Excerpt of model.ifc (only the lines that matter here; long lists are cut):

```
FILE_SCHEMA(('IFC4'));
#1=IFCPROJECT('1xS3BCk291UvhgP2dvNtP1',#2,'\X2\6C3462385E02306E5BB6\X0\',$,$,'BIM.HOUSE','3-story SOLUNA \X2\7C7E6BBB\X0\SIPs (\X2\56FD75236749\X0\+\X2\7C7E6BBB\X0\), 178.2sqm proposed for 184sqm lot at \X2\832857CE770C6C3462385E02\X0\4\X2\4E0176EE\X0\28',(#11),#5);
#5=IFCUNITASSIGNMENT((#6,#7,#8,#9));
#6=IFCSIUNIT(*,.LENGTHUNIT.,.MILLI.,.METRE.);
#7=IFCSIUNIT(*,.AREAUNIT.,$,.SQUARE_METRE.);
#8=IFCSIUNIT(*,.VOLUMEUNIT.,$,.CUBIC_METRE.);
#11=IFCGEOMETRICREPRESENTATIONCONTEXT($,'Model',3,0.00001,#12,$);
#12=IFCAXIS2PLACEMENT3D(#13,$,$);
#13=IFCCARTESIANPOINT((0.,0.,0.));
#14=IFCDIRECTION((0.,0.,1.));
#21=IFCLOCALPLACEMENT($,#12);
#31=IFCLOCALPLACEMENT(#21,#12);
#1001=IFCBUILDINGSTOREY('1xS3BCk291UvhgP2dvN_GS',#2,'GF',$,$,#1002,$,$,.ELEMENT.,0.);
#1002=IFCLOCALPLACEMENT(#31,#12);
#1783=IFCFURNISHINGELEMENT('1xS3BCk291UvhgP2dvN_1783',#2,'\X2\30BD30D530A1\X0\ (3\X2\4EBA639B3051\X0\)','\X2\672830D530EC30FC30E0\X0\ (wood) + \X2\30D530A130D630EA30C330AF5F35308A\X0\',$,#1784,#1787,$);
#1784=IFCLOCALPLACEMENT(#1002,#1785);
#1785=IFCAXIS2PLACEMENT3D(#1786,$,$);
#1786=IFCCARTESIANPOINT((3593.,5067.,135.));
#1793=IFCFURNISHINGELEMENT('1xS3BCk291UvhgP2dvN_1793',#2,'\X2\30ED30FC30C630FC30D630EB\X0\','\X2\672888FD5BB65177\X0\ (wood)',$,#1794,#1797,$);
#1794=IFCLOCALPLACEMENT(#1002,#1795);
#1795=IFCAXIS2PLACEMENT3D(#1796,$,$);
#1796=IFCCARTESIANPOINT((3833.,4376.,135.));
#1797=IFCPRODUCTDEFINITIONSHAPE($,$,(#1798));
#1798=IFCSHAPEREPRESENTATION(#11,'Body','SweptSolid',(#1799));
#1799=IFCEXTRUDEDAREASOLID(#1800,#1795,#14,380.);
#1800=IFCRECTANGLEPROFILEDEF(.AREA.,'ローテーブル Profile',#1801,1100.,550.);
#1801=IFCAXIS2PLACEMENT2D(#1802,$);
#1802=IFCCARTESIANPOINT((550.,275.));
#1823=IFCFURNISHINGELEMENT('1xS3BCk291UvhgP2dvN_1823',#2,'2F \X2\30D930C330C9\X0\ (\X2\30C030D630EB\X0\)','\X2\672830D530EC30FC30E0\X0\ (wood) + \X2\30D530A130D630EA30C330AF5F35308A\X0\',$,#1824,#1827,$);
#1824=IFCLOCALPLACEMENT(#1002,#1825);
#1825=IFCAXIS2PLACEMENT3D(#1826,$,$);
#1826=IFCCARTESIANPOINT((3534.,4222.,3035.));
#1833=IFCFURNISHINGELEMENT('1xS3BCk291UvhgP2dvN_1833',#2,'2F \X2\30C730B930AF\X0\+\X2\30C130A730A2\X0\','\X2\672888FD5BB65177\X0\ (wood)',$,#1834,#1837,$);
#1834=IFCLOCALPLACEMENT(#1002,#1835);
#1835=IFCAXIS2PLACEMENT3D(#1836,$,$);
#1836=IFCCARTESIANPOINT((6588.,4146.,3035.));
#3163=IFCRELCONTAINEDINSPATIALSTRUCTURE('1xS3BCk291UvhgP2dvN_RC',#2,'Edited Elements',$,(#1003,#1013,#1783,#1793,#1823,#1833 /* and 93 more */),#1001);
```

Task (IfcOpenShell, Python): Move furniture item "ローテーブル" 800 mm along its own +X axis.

```python
import ifcopenshell
import ifcopenshell.api.geometry
import ifcopenshell.util.placement
import ifcopenshell.util.unit

model = ifcopenshell.open("model.ifc")
unit_scale = ifcopenshell.util.unit.calculate_unit_scale(model)

item = model.by_guid("1xS3BCk291UvhgP2dvN_1793")
matrix = ifcopenshell.util.placement.get_local_placement(item.ObjectPlacement)
matrix[:3, 3] += matrix[:3, 0] * 0.8 / unit_scale
ifcopenshell.api.geometry.edit_object_placement(model, product=item, matrix=matrix, is_si=False)

print(ifcopenshell.util.placement.get_local_placement(item.ObjectPlacement).round(3) + 0.0)

model.write("model_edited.ifc")
```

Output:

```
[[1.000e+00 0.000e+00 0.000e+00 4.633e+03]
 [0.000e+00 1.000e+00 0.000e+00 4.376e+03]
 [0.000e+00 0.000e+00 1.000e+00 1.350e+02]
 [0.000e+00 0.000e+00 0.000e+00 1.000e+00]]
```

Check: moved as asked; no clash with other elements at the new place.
